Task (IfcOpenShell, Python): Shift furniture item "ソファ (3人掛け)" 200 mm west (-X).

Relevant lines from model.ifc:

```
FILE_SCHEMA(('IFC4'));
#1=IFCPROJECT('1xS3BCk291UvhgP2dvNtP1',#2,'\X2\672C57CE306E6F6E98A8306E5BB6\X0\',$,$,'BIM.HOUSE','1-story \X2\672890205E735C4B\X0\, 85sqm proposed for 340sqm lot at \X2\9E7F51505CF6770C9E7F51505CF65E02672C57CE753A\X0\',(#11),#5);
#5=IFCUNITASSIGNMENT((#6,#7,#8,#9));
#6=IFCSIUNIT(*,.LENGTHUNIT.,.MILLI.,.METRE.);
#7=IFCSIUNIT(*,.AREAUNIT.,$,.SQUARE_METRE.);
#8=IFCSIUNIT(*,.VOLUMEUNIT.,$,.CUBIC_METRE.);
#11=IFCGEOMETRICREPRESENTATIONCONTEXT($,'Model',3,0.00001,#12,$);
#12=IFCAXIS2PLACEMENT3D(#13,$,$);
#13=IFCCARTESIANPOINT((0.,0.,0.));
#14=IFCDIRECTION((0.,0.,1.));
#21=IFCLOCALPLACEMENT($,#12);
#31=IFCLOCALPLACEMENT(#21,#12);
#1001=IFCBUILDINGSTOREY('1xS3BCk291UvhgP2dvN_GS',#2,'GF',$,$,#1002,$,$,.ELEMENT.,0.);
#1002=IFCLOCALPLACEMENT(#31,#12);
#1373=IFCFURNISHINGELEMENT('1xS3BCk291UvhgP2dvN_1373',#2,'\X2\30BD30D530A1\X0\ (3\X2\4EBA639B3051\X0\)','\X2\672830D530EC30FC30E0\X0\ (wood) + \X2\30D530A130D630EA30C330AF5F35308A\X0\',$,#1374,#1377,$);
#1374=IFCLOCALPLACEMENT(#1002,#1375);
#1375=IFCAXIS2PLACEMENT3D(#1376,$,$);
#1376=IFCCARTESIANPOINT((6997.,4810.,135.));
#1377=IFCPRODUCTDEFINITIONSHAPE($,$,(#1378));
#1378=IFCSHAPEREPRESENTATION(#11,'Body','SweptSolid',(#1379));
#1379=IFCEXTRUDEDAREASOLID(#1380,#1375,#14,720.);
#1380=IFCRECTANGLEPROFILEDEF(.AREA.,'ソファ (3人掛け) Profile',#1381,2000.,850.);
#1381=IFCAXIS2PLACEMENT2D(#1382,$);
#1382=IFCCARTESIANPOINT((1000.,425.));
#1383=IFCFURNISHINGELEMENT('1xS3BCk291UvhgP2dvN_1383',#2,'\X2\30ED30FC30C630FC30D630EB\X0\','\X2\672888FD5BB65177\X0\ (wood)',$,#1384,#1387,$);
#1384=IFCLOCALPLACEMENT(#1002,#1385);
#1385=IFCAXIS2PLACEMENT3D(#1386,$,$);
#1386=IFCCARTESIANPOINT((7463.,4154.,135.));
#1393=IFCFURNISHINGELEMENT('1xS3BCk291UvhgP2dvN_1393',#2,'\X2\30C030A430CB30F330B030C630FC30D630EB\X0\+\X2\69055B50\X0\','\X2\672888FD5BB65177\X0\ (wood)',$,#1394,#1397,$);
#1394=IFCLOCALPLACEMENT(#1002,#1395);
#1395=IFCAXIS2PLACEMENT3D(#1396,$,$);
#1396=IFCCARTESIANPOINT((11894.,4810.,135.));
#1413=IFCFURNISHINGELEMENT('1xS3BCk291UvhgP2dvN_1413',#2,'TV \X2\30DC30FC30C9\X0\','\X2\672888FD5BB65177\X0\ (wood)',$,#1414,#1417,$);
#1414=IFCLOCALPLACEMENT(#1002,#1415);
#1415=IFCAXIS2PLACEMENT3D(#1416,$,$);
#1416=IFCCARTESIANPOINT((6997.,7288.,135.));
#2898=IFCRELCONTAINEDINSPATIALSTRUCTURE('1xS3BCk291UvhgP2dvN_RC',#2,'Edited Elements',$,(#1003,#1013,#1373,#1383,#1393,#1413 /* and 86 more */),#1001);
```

```python
import ifcopenshell
import ifcopenshell.api.geometry
import ifcopenshell.util.placement

model = ifcopenshell.open("model.ifc")

item = model.by_id(1373)
matrix = ifcopenshell.util.placement.get_local_placement(item.ObjectPlacement)
matrix[0, 3] -= 200.0
ifcopenshell.api.geometry.edit_object_placement(model, product=item, matrix=matrix, is_si=False)

print(ifcopenshell.util.placement.get_local_placement(item.ObjectPlacement).round(3) + 0.0)

model.write("model_updated.ifc")
```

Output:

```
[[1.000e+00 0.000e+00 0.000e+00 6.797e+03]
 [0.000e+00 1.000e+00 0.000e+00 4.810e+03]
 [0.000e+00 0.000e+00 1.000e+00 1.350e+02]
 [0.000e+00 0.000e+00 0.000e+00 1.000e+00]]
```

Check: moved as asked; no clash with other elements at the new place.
